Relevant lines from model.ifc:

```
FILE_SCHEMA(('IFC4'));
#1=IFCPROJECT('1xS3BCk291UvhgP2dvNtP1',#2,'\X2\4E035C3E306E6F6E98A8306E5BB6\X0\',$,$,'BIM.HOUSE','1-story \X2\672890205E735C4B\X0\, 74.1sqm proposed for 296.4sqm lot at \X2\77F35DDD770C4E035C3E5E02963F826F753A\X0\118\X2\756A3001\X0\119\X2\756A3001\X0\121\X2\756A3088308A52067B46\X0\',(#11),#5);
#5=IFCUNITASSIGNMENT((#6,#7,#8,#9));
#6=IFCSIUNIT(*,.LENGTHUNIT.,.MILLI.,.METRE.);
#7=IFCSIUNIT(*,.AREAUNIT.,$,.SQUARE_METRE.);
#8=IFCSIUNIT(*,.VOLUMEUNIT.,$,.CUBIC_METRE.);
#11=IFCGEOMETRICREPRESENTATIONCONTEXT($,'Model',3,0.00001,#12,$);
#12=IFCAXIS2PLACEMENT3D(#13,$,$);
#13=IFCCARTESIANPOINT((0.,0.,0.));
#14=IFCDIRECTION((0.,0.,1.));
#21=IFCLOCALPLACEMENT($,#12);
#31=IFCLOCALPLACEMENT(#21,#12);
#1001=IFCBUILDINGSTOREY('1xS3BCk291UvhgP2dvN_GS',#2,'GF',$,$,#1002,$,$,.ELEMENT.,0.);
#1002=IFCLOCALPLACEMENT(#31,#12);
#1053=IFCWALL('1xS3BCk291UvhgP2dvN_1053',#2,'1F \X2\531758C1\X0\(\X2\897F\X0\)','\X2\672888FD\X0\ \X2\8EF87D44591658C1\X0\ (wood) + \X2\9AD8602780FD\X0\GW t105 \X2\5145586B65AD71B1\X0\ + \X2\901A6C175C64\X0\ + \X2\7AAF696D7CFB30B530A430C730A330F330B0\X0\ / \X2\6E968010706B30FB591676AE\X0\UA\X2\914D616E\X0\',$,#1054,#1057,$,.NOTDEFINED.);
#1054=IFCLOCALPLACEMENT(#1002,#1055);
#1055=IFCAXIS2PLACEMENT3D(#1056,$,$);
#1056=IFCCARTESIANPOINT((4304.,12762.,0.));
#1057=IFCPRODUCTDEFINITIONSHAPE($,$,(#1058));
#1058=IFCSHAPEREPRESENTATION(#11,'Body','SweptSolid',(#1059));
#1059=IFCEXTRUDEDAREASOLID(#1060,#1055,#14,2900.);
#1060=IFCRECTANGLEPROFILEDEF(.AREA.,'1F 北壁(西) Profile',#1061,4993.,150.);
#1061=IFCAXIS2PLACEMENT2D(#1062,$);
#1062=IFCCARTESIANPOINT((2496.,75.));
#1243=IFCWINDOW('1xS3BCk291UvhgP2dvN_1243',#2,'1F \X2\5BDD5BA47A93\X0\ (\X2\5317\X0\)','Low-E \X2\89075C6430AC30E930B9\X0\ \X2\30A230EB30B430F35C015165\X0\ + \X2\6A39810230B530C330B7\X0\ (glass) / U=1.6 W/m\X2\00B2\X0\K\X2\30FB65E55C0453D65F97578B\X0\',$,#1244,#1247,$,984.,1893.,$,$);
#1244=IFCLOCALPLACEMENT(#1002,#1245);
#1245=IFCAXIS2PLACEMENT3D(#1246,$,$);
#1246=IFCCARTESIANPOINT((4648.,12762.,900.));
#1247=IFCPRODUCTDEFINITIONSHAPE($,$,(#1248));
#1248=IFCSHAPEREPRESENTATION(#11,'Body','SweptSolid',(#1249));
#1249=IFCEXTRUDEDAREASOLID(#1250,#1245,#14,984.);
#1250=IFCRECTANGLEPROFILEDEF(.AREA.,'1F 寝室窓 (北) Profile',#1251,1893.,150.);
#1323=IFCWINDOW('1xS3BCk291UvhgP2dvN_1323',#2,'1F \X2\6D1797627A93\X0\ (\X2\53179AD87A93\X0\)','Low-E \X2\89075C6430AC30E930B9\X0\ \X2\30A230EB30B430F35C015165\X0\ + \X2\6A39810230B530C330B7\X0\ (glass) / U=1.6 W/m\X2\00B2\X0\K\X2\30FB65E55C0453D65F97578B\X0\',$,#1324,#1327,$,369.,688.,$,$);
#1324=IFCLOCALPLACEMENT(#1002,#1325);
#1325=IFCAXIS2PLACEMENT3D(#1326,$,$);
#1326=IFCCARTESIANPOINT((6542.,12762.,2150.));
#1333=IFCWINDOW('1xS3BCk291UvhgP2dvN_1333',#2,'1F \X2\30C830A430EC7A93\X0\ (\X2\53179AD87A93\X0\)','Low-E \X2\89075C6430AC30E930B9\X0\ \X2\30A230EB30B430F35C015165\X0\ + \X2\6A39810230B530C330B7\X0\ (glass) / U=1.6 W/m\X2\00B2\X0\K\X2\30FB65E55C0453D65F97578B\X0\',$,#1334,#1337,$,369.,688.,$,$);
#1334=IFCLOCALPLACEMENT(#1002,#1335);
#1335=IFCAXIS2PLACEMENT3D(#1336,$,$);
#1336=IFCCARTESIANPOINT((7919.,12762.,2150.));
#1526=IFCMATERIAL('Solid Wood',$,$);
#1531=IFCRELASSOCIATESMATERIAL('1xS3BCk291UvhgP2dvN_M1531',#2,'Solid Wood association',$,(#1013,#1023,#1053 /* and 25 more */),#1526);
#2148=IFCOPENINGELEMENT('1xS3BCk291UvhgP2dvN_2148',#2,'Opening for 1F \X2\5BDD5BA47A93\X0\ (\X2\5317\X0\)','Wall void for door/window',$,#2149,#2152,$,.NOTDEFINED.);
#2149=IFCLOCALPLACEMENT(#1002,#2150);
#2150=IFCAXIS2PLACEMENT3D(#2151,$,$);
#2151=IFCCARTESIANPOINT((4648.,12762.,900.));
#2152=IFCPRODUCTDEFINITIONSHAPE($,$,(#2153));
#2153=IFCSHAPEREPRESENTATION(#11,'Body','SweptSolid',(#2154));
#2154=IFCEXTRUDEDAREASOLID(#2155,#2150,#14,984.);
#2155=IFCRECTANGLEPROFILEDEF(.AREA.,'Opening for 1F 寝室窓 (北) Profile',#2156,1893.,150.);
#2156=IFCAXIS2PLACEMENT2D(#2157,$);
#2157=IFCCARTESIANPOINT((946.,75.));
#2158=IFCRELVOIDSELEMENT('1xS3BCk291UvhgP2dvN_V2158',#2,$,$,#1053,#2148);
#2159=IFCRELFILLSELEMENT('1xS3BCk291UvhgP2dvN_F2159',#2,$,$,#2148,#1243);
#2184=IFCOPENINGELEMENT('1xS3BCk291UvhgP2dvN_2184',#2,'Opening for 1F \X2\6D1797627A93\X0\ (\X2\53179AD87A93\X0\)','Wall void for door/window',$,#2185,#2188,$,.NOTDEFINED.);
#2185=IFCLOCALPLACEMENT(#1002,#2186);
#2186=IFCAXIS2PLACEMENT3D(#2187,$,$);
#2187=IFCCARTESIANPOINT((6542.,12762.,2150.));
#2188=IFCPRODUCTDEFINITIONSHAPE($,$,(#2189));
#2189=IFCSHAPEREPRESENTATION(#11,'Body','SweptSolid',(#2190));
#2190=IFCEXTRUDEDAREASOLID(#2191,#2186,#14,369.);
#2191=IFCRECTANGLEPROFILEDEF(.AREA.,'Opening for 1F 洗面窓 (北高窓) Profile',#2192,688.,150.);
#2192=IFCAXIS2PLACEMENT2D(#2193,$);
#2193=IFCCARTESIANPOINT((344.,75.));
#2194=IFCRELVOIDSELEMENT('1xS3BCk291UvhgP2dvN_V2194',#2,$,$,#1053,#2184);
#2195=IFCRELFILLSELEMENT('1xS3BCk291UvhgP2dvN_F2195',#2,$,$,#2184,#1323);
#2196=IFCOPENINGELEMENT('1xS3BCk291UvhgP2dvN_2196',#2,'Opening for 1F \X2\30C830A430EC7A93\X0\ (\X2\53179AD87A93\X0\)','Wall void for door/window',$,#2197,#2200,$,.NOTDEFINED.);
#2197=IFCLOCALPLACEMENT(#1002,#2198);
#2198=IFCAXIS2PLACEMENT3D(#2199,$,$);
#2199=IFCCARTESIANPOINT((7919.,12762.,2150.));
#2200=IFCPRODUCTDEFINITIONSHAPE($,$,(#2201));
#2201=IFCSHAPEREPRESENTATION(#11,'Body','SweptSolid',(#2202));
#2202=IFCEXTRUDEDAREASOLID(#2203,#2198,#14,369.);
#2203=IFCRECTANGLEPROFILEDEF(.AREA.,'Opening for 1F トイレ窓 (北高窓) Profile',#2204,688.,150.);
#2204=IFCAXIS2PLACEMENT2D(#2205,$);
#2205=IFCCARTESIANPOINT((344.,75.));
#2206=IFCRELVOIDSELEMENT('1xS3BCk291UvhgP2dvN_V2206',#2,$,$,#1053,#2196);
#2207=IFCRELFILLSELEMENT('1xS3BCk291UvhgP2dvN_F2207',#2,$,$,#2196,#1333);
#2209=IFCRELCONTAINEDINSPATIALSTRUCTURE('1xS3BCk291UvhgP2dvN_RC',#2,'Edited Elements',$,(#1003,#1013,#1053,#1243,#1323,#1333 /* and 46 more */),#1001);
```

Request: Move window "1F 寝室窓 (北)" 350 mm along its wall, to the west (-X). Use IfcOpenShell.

```python
import ifcopenshell
import ifcopenshell.api.geometry
import ifcopenshell.util.placement

model = ifcopenshell.open("model.ifc")

window = model.by_guid("1xS3BCk291UvhgP2dvN_1243")
opening = window.FillsVoids[0].RelatingOpeningElement
wall = opening.VoidsElements[0].RelatingBuildingElement

wall_matrix = ifcopenshell.util.placement.get_local_placement(wall.ObjectPlacement)
shift = wall_matrix[:3, 0] * -350.0
before = ifcopenshell.util.placement.get_local_placement(window.ObjectPlacement)[:3, 3].copy()

# The window is not placed relative to its opening, so move both.
for product in (opening, window):
    matrix = ifcopenshell.util.placement.get_local_placement(product.ObjectPlacement)
    matrix[:3, 3] += shift
    ifcopenshell.api.geometry.edit_object_placement(model, product=product, matrix=matrix, is_si=False)

after = ifcopenshell.util.placement.get_local_placement(window.ObjectPlacement)[:3, 3]
print("window moved by", (after - before).round(3) + 0.0)

model.write("model-out.ifc")
```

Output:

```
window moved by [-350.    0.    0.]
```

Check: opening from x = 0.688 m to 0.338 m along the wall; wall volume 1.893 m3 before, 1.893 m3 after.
